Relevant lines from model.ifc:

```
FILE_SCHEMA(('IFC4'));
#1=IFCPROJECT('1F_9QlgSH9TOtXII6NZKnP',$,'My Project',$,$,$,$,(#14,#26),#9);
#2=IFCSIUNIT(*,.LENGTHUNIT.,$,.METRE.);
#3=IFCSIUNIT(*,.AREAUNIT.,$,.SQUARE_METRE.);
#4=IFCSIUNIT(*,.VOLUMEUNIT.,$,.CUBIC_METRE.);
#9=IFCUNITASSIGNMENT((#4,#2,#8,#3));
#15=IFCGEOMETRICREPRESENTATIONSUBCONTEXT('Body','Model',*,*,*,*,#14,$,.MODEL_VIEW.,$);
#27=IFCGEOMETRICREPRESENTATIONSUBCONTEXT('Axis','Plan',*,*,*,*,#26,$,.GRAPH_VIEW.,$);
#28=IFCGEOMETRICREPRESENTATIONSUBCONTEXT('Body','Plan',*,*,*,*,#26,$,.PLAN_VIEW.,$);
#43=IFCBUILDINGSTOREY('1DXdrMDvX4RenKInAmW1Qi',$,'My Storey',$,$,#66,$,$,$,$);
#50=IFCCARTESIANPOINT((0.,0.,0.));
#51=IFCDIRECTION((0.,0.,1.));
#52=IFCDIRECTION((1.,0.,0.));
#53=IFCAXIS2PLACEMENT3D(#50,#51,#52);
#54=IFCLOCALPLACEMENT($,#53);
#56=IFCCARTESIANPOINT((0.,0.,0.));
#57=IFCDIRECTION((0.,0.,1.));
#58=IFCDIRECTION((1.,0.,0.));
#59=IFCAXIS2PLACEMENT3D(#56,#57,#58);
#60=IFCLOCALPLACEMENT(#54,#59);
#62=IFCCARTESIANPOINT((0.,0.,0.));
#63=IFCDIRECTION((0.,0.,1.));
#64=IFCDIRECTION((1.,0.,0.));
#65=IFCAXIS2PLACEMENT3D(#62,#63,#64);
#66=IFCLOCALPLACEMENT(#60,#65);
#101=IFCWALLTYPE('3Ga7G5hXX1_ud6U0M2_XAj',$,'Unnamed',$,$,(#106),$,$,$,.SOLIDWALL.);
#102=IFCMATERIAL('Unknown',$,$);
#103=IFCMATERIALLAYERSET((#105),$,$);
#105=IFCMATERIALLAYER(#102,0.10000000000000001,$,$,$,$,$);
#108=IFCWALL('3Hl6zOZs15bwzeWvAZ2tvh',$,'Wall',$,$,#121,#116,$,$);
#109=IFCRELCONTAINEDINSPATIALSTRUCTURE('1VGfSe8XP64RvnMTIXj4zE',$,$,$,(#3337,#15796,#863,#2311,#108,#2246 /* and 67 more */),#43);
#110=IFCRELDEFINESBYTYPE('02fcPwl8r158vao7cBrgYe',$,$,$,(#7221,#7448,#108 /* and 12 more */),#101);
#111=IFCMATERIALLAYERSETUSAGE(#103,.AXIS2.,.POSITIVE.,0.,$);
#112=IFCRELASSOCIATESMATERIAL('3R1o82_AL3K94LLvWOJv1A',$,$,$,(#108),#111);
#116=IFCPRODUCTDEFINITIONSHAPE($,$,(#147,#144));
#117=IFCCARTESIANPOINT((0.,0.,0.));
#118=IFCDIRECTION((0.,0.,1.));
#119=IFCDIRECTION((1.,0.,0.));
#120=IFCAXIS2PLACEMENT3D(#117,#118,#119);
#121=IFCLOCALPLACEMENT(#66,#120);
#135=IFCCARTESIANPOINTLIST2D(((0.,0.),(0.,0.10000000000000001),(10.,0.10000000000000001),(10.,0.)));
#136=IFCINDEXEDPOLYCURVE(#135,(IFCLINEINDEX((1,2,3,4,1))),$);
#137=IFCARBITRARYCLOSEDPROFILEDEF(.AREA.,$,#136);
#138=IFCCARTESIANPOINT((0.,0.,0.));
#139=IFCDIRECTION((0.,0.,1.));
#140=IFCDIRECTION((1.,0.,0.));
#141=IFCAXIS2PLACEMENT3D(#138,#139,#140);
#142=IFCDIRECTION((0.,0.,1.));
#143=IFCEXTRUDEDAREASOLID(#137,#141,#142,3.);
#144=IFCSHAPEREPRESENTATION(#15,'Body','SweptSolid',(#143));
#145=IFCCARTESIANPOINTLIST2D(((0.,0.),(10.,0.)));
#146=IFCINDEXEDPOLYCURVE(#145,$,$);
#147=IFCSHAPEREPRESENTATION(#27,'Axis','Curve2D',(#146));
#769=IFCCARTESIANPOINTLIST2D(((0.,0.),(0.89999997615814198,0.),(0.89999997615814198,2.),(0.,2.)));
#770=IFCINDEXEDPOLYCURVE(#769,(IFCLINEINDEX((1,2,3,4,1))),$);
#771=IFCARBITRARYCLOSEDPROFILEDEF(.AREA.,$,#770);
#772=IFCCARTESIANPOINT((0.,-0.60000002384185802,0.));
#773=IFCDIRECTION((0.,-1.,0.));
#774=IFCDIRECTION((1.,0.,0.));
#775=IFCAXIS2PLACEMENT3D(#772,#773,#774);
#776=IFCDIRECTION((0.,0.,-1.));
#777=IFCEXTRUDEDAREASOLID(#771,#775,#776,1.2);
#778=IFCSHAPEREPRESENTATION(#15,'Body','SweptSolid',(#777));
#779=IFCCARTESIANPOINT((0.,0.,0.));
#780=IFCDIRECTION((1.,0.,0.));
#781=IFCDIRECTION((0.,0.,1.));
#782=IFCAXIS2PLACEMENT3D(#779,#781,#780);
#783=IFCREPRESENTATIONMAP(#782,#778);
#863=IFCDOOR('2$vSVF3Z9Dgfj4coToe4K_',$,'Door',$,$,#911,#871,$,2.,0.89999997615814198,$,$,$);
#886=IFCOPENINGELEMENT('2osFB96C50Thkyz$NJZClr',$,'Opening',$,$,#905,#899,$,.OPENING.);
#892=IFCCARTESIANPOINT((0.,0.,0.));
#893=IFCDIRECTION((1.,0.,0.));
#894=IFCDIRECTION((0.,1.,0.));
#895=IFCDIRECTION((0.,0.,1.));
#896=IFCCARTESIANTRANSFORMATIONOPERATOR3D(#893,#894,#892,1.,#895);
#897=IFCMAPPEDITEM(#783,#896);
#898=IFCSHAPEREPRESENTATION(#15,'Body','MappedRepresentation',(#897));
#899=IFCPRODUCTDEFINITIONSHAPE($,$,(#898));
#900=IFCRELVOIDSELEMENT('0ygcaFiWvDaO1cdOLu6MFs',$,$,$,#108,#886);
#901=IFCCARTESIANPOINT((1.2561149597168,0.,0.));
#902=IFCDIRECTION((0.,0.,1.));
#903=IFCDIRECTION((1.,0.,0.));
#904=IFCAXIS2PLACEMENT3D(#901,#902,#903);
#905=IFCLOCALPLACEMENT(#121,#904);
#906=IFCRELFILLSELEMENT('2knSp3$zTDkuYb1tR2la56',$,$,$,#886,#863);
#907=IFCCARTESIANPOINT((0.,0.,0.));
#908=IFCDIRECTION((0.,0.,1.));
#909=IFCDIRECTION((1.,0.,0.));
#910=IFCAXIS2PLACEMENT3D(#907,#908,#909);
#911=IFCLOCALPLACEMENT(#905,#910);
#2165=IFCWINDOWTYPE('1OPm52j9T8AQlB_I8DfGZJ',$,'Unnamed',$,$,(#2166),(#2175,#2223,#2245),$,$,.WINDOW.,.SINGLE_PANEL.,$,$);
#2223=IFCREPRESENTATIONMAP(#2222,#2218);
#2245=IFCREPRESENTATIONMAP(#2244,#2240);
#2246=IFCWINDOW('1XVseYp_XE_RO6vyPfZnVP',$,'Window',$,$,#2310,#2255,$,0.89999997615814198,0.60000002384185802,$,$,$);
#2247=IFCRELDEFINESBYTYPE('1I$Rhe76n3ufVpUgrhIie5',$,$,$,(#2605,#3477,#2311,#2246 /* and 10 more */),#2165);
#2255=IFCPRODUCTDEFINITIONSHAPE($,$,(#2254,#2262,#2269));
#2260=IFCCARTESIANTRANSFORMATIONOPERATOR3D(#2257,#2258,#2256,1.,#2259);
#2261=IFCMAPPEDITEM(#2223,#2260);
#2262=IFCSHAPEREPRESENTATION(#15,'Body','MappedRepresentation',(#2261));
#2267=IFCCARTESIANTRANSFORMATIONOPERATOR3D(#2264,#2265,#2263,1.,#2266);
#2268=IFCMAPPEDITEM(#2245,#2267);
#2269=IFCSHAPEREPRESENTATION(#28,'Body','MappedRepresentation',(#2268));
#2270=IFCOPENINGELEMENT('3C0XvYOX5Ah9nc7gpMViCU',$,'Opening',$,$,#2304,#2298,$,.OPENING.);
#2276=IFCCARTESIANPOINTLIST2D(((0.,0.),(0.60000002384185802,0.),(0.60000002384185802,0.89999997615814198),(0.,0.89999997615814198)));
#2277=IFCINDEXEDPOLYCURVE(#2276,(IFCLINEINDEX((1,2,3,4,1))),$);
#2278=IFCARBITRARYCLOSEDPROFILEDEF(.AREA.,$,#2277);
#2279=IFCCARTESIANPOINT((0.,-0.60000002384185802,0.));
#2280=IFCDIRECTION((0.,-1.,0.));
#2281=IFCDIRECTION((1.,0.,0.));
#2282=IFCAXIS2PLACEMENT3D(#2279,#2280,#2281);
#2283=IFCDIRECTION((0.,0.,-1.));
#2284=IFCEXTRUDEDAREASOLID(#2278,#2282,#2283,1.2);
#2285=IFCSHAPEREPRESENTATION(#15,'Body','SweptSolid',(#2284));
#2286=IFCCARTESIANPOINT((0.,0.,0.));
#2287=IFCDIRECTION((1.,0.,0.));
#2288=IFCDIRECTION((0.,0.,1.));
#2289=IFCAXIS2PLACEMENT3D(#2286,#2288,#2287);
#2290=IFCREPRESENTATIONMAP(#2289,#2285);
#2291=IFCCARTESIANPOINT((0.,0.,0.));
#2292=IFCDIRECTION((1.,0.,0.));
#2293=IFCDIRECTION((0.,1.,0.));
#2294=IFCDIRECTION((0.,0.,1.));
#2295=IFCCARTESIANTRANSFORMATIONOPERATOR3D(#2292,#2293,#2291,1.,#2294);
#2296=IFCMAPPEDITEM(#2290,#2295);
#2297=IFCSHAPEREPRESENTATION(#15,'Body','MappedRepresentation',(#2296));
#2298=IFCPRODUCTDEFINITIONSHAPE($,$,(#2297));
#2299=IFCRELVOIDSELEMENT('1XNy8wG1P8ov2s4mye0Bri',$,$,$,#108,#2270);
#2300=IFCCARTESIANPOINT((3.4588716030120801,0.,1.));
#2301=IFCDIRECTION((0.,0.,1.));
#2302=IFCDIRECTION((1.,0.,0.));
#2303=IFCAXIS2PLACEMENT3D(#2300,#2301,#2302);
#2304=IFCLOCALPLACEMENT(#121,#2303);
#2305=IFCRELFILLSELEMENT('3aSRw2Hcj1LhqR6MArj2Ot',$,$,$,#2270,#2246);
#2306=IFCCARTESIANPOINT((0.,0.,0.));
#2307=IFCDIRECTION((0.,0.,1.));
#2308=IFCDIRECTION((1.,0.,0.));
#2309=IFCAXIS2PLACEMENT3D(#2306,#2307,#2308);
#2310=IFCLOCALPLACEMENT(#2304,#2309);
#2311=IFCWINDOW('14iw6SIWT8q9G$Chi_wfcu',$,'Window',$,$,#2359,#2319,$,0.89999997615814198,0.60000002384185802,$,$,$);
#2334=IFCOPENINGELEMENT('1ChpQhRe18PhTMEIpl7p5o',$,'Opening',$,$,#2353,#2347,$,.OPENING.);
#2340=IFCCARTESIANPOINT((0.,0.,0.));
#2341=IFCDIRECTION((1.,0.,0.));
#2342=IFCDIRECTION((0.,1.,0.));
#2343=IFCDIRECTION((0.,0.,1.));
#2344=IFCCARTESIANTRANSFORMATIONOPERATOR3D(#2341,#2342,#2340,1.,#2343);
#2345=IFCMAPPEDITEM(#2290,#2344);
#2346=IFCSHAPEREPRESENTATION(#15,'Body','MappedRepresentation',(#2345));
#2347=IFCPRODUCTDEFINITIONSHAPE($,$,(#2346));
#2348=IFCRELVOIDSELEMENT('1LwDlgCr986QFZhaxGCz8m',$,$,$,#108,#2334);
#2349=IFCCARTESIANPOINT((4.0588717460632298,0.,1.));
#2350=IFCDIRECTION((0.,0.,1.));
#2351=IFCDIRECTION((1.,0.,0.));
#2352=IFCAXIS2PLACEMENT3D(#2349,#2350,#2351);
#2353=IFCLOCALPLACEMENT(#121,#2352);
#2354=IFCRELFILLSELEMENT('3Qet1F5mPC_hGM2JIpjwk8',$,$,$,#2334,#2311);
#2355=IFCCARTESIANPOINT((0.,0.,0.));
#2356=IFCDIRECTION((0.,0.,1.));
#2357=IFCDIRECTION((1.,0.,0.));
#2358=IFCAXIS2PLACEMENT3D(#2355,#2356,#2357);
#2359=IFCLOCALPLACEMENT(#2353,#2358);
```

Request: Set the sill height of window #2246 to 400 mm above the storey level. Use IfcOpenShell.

```python
import numpy as np
import ifcopenshell
import ifcopenshell.api.geometry
import ifcopenshell.geom
import ifcopenshell.util.element
import ifcopenshell.util.placement
import ifcopenshell.util.shape
import ifcopenshell.util.unit

model = ifcopenshell.open("model.ifc")
unit_scale = ifcopenshell.util.unit.calculate_unit_scale(model)

window = model.by_guid("1XVseYp_XE_RO6vyPfZnVP")
opening = window.FillsVoids[0].RelatingOpeningElement
storey = ifcopenshell.util.element.get_container(window, ifc_class="IfcBuildingStorey")
level = ifcopenshell.util.placement.get_local_placement(storey.ObjectPlacement)[2, 3]

# The opening's origin need not be at the sill, so measure its lowest point.
shape = ifcopenshell.geom.create_shape(ifcopenshell.geom.settings(), opening)
bottom = ifcopenshell.util.shape.get_shape_bottom_elevation(shape, shape.geometry) / unit_scale
dz = level + 0.4 / unit_scale - bottom

shift = np.array([0.0, 0.0, dz])
# The window is placed relative to its opening, so it follows when the opening moves.
matrix = ifcopenshell.util.placement.get_local_placement(opening.ObjectPlacement)
matrix[:3, 3] += shift
ifcopenshell.api.geometry.edit_object_placement(
    model, product=opening, matrix=matrix, is_si=False, should_transform_children=True
)

print(f"moved by {dz * unit_scale:+.3f} m")

model.write("model_edited.ifc")
```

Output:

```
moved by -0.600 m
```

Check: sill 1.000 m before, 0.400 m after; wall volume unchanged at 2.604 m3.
